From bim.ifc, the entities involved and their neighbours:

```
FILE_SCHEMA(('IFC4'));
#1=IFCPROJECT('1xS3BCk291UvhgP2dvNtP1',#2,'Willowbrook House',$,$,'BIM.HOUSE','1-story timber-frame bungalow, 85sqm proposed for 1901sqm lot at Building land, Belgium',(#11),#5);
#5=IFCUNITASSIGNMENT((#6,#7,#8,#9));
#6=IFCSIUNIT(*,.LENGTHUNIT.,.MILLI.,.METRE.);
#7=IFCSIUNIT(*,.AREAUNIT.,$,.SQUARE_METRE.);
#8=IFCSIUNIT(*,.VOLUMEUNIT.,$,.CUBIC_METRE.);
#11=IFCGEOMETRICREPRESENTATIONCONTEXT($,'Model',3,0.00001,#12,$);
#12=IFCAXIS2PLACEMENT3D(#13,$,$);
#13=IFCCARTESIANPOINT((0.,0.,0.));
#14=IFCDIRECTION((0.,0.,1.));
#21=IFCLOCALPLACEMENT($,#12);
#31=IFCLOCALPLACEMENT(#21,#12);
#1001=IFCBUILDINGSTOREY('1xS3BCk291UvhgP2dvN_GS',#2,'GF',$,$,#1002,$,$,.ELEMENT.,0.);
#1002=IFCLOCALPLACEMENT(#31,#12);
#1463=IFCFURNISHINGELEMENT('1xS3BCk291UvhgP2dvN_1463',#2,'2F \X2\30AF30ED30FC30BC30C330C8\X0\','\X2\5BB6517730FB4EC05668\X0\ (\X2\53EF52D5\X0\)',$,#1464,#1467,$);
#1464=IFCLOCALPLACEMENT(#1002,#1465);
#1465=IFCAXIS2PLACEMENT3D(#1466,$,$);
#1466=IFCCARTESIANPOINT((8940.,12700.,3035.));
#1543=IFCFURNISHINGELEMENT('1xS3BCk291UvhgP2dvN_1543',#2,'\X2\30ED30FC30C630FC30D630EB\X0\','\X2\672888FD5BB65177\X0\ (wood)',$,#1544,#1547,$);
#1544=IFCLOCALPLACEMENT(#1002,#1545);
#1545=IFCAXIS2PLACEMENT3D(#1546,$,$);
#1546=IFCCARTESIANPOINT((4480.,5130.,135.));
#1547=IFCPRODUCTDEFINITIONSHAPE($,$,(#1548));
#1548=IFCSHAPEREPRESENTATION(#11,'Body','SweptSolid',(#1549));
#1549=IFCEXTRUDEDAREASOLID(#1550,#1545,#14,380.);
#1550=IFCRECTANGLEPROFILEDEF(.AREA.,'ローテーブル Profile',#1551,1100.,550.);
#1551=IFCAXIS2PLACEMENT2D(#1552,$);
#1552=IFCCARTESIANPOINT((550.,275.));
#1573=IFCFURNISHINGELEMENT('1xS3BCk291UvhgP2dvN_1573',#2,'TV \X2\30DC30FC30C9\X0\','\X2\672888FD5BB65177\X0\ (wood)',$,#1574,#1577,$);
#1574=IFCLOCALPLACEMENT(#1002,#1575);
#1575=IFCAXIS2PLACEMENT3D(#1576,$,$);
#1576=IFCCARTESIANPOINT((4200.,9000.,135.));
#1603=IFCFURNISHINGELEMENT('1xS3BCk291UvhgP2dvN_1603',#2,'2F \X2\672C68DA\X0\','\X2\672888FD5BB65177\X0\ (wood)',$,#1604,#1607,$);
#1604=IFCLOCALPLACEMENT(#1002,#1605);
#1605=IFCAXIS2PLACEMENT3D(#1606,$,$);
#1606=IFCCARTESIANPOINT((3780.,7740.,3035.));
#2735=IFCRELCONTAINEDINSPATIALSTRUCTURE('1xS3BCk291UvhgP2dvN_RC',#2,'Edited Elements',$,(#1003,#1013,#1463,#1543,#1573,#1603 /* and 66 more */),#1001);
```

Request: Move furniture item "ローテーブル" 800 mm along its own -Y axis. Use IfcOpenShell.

```python
import ifcopenshell
import ifcopenshell.api.geometry
import ifcopenshell.util.placement
import ifcopenshell.util.unit

model = ifcopenshell.open("bim.ifc")
unit_scale = ifcopenshell.util.unit.calculate_unit_scale(model)

item = model.by_guid("1xS3BCk291UvhgP2dvN_1543")
matrix = ifcopenshell.util.placement.get_local_placement(item.ObjectPlacement)
matrix[:3, 3] -= matrix[:3, 1] * 0.8 / unit_scale
ifcopenshell.api.geometry.edit_object_placement(model, product=item, matrix=matrix, is_si=False)

print(ifcopenshell.util.placement.get_local_placement(item.ObjectPlacement).round(3) + 0.0)

model.write("bim-out.ifc")
```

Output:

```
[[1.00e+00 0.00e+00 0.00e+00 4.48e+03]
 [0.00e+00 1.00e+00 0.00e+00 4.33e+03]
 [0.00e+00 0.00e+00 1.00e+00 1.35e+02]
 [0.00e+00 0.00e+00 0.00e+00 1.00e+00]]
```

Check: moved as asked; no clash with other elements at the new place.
